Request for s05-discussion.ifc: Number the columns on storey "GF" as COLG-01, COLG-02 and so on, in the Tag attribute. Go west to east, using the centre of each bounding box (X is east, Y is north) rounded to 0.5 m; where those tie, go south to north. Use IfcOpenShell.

First a look at what the model holds.

```python
import ifcopenshell
import ifcopenshell.util.element
import ifcopenshell.util.placement

model = ifcopenshell.open("s05-discussion.ifc")
print(model.schema)
storey = next(s for s in model.by_type("IfcBuildingStorey") if s.Name == "GF")
columns = [e for e in ifcopenshell.util.element.get_decomposition(storey) if e.is_a("IfcColumn")]
for e in sorted(columns, key=lambda e: e.id()):
    origin = ifcopenshell.util.placement.get_local_placement(e.ObjectPlacement)[:3, 3]
    print(e.id(), e.Tag, e.Name, origin.round(2) + 0.0, sep=" | ")
```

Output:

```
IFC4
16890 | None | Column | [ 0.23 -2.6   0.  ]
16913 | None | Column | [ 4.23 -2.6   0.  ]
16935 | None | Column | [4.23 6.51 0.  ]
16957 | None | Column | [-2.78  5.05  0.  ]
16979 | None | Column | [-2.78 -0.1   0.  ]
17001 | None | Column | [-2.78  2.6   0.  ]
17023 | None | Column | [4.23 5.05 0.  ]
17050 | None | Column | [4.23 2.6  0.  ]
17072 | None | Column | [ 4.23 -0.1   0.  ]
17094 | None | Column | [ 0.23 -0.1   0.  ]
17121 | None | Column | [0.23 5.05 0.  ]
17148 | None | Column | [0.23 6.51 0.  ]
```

```python
import ifcopenshell
import ifcopenshell.geom
import ifcopenshell.util.element
import ifcopenshell.util.shape

model = ifcopenshell.open("s05-discussion.ifc")
settings = ifcopenshell.geom.settings()
settings.set("use-world-coords", True)


def centre(element):
    shape = ifcopenshell.geom.create_shape(settings, element)
    return ifcopenshell.util.shape.get_bbox_centroid(shape.geometry)


storey = next(s for s in model.by_type("IfcBuildingStorey") if s.Name == "GF")
columns = [e for e in ifcopenshell.util.element.get_decomposition(storey) if e.is_a("IfcColumn")]

# Insertion points can sit at a corner or the storey origin, so sort by the geometry (in metres).
centres = {e: centre(e) for e in columns}
columns.sort(key=lambda e: (round(centres[e][0] / 0.5), centres[e][1]))

for i, e in enumerate(columns, start=1):
    number = f"COLG-{i:02d}"
    e.Tag = number
    print(e.id(), number)

model.write("s05-discussion_v2.ifc")
```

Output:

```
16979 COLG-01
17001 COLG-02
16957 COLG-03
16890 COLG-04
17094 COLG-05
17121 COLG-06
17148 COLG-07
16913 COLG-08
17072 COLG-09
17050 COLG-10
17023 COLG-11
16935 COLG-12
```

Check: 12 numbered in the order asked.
